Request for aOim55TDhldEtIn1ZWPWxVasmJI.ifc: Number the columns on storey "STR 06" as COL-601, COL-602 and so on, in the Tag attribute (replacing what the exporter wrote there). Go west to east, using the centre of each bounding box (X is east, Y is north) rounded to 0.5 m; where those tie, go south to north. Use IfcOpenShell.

First a look at what the model holds.

```python
import ifcopenshell
import ifcopenshell.util.element
import ifcopenshell.util.placement

model = ifcopenshell.open("aOim55TDhldEtIn1ZWPWxVasmJI.ifc")
print(model.schema)
storey = next(s for s in model.by_type("IfcBuildingStorey") if s.Name == "STR 06")
columns = [e for e in ifcopenshell.util.element.get_decomposition(storey) if e.is_a("IfcColumn")]
for e in sorted(columns, key=lambda e: e.id()):
    origin = ifcopenshell.util.placement.get_local_placement(e.ObjectPlacement)[:3, 3]
    print(e.id(), e.Tag, e.Name, origin.round(2) + 0.0, sep=" | ")
```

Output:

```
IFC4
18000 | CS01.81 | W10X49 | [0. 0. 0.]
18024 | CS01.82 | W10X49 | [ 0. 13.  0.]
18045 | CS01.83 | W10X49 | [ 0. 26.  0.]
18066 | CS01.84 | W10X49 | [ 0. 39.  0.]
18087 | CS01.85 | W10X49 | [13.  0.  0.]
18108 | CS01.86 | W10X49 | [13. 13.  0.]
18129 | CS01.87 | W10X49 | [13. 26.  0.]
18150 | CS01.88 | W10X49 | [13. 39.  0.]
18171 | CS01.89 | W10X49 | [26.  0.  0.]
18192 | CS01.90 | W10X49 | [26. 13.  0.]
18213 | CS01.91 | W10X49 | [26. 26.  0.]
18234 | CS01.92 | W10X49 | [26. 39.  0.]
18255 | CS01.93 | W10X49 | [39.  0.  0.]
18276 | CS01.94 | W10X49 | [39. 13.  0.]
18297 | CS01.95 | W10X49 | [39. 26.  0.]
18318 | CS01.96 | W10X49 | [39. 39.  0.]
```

```python
import ifcopenshell
import ifcopenshell.geom
import ifcopenshell.util.element
import ifcopenshell.util.shape

model = ifcopenshell.open("aOim55TDhldEtIn1ZWPWxVasmJI.ifc")
settings = ifcopenshell.geom.settings()
settings.set("use-world-coords", True)


def centre(element):
    shape = ifcopenshell.geom.create_shape(settings, element)
    return ifcopenshell.util.shape.get_bbox_centroid(shape.geometry)


storey = next(s for s in model.by_type("IfcBuildingStorey") if s.Name == "STR 06")
columns = [e for e in ifcopenshell.util.element.get_decomposition(storey) if e.is_a("IfcColumn")]

# Insertion points can sit at a corner or the storey origin, so sort by the geometry (in metres).
centres = {e: centre(e) for e in columns}
columns.sort(key=lambda e: (round(centres[e][0] / 0.5), centres[e][1]))

for i, e in enumerate(columns, start=1):
    number = f"COL-6{i:02d}"
    e.Tag = number
    print(e.id(), number)

model.write("aOim55TDhldEtIn1ZWPWxVasmJI_edited.ifc")
```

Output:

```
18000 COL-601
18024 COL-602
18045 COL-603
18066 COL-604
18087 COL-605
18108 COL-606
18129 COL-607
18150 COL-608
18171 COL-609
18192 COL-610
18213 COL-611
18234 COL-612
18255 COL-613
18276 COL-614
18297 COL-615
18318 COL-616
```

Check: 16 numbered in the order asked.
